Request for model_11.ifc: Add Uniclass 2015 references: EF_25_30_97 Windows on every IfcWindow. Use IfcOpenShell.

First a look at what the model holds.

```python
import ifcopenshell

model = ifcopenshell.open("model_11.ifc")
print(model.schema)
print("classifications:", [c.Name for c in model.by_type("IfcClassification")])
for ifc_class in ("IfcDoor", "IfcRoof", "IfcStair", "IfcWall", "IfcWindow"):
    print(ifc_class, len(model.by_type(ifc_class)))
```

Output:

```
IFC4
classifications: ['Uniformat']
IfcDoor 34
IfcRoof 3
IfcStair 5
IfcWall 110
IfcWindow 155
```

```python
import ifcopenshell
import ifcopenshell.api.classification

model = ifcopenshell.open("model_11.ifc")

system = ifcopenshell.api.classification.add_classification(model, classification="Uniclass 2015")

codes = {
    "IfcWindow": ("EF_25_30_97", "Windows"),
}
for ifc_class, (code, name) in codes.items():
    products = model.by_type(ifc_class)
    ifcopenshell.api.classification.add_reference(
        model, products=products, classification=system, identification=code, name=name
    )
    print(code, len(products))

model.write("model_11-out.ifc")
```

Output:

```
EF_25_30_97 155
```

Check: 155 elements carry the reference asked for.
